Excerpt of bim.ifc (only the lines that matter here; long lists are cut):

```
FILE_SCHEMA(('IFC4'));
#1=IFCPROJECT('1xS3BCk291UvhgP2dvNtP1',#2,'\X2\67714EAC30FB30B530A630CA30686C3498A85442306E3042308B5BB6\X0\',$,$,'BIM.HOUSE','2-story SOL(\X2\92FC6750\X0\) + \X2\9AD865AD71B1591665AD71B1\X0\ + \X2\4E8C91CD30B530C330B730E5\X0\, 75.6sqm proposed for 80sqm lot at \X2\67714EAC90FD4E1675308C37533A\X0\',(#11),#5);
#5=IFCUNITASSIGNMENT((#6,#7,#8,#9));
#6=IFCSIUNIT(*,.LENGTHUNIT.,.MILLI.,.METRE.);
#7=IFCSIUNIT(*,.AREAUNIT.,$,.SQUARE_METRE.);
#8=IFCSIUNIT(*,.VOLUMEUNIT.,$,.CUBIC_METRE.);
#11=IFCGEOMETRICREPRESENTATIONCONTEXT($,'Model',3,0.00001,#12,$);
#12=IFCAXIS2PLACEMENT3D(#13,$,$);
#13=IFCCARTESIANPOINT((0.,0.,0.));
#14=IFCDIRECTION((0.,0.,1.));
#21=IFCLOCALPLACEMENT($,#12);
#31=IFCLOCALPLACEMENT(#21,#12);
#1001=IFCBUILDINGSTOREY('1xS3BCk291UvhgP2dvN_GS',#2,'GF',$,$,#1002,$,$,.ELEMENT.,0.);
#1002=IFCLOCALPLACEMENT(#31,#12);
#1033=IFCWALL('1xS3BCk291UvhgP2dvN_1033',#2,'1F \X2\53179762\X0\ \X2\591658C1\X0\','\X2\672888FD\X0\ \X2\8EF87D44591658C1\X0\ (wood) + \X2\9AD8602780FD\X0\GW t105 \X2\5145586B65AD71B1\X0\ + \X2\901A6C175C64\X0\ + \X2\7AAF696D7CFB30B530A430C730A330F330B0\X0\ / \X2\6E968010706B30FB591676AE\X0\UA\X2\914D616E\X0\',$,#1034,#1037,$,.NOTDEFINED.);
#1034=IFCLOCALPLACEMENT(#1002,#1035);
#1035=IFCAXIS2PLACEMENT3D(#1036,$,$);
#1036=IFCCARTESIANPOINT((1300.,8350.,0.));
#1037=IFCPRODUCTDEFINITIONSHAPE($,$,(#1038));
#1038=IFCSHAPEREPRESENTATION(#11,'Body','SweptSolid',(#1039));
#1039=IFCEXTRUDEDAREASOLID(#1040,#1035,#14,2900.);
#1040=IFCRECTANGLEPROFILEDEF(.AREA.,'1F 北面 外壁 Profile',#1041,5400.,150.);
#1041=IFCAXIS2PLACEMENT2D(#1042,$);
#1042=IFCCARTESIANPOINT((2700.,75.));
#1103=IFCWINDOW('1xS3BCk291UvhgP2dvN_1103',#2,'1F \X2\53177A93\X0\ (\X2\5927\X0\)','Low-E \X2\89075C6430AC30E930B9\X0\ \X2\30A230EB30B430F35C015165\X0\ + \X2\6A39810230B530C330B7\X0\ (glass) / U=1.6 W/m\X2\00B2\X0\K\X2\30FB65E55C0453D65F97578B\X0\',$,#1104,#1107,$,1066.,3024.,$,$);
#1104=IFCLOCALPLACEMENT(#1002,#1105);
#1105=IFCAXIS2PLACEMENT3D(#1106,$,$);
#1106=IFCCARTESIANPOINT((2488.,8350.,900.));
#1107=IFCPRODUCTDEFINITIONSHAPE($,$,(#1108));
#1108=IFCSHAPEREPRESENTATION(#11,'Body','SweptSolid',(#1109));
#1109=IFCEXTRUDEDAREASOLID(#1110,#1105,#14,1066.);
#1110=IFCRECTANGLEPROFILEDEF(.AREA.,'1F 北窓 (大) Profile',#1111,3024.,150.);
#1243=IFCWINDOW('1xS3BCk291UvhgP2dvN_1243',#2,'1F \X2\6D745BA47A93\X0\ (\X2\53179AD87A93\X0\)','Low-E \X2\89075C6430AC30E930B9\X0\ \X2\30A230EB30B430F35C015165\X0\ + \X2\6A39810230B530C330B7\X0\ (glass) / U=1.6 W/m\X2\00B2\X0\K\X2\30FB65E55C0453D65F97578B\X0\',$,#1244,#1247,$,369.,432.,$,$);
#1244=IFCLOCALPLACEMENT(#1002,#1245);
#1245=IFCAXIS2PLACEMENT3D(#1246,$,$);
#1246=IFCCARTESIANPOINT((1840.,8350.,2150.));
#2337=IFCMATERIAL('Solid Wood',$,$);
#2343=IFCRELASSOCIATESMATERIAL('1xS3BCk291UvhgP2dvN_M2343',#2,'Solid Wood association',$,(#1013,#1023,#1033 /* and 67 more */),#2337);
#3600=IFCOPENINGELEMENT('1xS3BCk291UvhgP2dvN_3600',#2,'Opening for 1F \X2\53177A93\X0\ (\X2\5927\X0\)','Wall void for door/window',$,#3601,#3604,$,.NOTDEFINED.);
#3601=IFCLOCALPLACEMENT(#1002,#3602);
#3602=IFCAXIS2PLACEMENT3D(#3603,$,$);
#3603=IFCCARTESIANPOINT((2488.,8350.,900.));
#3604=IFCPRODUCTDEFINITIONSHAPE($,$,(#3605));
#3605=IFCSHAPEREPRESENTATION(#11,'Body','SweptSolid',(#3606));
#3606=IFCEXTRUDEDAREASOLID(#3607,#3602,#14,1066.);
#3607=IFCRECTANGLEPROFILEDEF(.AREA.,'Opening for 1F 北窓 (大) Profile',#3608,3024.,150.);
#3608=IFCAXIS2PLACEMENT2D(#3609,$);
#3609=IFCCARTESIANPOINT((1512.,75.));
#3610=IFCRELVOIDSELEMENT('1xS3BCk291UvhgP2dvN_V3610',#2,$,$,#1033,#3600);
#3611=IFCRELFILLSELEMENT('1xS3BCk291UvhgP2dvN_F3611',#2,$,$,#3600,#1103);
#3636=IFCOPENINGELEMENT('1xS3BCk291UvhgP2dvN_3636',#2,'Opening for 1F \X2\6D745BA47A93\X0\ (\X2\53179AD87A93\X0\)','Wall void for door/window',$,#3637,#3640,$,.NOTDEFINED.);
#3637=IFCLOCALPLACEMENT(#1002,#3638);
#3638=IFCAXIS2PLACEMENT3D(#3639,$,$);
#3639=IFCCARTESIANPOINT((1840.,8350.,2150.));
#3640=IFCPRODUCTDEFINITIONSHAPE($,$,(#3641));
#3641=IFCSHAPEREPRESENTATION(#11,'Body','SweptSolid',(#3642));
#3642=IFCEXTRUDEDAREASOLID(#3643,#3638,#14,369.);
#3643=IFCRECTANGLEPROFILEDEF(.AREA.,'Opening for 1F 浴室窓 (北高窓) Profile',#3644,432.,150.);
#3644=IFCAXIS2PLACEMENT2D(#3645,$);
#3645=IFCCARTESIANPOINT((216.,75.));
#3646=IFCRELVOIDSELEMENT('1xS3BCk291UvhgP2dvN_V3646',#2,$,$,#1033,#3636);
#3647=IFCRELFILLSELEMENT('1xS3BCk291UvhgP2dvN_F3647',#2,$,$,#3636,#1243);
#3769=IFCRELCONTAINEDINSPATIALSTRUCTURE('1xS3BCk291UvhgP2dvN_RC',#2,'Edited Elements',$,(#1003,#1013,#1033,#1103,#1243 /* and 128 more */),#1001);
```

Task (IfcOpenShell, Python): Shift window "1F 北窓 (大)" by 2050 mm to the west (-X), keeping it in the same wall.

```python
import ifcopenshell
import ifcopenshell.api.geometry
import ifcopenshell.util.placement

model = ifcopenshell.open("bim.ifc")

window = model.by_id(1103)
opening = window.FillsVoids[0].RelatingOpeningElement
wall = opening.VoidsElements[0].RelatingBuildingElement

wall_matrix = ifcopenshell.util.placement.get_local_placement(wall.ObjectPlacement)
shift = wall_matrix[:3, 0] * -2050.0
before = ifcopenshell.util.placement.get_local_placement(window.ObjectPlacement)[:3, 3].copy()

# The window is not placed relative to its opening, so move both.
for product in (opening, window):
    matrix = ifcopenshell.util.placement.get_local_placement(product.ObjectPlacement)
    matrix[:3, 3] += shift
    ifcopenshell.api.geometry.edit_object_placement(model, product=product, matrix=matrix, is_si=False)

after = ifcopenshell.util.placement.get_local_placement(window.ObjectPlacement)[:3, 3]
print("window moved by", (after - before).round(3) + 0.0)

model.write("bim-out.ifc")
```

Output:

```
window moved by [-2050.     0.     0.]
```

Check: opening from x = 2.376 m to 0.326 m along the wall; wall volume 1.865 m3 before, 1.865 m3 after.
